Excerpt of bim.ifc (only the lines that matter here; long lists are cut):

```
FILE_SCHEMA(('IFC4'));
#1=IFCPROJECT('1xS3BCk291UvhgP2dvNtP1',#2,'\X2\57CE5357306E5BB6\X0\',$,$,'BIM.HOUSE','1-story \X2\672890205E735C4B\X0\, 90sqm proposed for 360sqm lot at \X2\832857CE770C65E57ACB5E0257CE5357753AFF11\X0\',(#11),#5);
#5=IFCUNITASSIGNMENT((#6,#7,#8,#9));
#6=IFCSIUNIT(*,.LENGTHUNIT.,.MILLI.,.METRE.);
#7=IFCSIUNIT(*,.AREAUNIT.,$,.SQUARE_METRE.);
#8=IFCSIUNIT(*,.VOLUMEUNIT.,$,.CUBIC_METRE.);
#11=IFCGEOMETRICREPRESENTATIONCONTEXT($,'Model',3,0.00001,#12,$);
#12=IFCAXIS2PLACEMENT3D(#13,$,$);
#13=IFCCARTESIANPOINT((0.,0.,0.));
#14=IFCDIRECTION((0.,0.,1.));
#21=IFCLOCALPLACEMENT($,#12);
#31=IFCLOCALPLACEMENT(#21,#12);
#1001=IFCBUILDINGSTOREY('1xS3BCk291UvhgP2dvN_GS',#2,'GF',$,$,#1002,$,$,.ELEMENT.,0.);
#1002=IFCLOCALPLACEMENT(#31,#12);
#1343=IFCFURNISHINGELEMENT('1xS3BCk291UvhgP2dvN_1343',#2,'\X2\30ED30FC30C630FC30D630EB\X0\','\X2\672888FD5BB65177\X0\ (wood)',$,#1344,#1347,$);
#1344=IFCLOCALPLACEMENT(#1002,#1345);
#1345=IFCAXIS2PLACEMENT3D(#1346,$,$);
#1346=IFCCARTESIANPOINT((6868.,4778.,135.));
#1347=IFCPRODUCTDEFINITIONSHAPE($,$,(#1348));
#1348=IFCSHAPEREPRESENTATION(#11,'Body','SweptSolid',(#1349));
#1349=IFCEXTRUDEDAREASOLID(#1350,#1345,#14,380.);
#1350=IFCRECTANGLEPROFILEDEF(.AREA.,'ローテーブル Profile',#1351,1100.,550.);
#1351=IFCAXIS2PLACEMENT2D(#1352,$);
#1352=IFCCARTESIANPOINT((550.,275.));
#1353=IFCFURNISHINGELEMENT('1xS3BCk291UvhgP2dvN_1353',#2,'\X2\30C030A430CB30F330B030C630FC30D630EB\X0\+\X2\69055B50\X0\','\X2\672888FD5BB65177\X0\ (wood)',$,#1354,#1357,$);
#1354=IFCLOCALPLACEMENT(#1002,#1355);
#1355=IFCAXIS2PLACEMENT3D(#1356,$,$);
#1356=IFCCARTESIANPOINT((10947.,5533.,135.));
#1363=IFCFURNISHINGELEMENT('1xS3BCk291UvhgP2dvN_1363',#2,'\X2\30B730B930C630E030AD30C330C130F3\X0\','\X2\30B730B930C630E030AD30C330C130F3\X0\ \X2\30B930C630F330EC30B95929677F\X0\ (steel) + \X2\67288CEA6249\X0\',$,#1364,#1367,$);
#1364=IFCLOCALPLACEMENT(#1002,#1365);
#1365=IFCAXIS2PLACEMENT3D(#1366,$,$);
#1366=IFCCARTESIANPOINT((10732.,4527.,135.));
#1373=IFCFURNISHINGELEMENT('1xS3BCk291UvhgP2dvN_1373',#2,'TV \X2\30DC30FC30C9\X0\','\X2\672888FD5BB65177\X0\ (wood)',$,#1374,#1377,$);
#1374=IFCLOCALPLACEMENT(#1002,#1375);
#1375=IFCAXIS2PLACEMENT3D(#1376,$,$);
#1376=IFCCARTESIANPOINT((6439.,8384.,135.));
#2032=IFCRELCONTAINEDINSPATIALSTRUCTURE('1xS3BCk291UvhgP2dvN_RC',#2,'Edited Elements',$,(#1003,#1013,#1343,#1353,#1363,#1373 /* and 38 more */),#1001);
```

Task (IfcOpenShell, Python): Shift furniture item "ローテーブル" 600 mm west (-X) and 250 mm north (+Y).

```python
import ifcopenshell
import ifcopenshell.api.geometry
import ifcopenshell.util.placement

model = ifcopenshell.open("bim.ifc")

item = model.by_guid("1xS3BCk291UvhgP2dvN_1343")
matrix = ifcopenshell.util.placement.get_local_placement(item.ObjectPlacement)
matrix[0, 3] -= 600.0
matrix[1, 3] += 250.0
ifcopenshell.api.geometry.edit_object_placement(model, product=item, matrix=matrix, is_si=False)

print(ifcopenshell.util.placement.get_local_placement(item.ObjectPlacement).round(3) + 0.0)

model.write("bim_updated.ifc")
```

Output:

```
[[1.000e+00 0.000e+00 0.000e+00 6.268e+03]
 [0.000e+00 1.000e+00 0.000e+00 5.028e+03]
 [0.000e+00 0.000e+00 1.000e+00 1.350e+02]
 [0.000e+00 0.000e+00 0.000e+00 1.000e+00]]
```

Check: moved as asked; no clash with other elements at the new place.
